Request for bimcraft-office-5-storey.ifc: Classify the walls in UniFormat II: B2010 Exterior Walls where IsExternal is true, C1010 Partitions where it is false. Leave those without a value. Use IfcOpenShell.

First a look at what the model holds.

```python
import ifcopenshell
import ifcopenshell.util.element

model = ifcopenshell.open("bimcraft-office-5-storey.ifc")
print(model.schema)
print("classifications:", [c.Name for c in model.by_type("IfcClassification")])
values = [ifcopenshell.util.element.get_pset(e, "Pset_WallCommon", "IsExternal") for e in model.by_type("IfcWall")]
for value in (True, False, None):
    print("IsExternal", value, values.count(value))
```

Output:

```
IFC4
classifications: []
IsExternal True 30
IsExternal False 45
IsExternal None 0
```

```python
import ifcopenshell
import ifcopenshell.api.classification
import ifcopenshell.util.element

model = ifcopenshell.open("bimcraft-office-5-storey.ifc")

system = ifcopenshell.api.classification.add_classification(model, classification="UniFormat II")

walls = model.by_type("IfcWall")
external = {e: ifcopenshell.util.element.get_pset(e, "Pset_WallCommon", "IsExternal") for e in walls}
for flag, code, name in ((True, "B2010", "Exterior Walls"), (False, "C1010", "Partitions")):
    products = [e for e in walls if external[e] is flag]
    ifcopenshell.api.classification.add_reference(
        model, products=products, classification=system, identification=code, name=name
    )
    print(code, len(products))

model.write("bimcraft-office-5-storey_edited.ifc")
```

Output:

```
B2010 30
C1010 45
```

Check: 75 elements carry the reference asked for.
